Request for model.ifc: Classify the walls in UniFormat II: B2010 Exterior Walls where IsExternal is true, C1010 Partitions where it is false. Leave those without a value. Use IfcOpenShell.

First a look at what the model holds.

```python
import ifcopenshell
import ifcopenshell.util.element

model = ifcopenshell.open("model.ifc")
print(model.schema)
print("classifications:", [c.Name for c in model.by_type("IfcClassification")])
values = [ifcopenshell.util.element.get_pset(e, "Pset_WallCommon", "IsExternal") for e in model.by_type("IfcWall")]
for value in (True, False, None):
    print("IsExternal", value, values.count(value))
```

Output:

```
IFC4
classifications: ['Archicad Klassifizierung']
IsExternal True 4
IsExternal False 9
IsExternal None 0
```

```python
import ifcopenshell
import ifcopenshell.api.classification
import ifcopenshell.util.element

model = ifcopenshell.open("model.ifc")

system = ifcopenshell.api.classification.add_classification(model, classification="UniFormat II")

walls = model.by_type("IfcWall")
external = {e: ifcopenshell.util.element.get_pset(e, "Pset_WallCommon", "IsExternal") for e in walls}
for flag, code, name in ((True, "B2010", "Exterior Walls"), (False, "C1010", "Partitions")):
    products = [e for e in walls if external[e] is flag]
    ifcopenshell.api.classification.add_reference(
        model, products=products, classification=system, identification=code, name=name
    )
    print(code, len(products))

model.write("model_rev.ifc")
```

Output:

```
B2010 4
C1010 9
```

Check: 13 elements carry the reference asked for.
